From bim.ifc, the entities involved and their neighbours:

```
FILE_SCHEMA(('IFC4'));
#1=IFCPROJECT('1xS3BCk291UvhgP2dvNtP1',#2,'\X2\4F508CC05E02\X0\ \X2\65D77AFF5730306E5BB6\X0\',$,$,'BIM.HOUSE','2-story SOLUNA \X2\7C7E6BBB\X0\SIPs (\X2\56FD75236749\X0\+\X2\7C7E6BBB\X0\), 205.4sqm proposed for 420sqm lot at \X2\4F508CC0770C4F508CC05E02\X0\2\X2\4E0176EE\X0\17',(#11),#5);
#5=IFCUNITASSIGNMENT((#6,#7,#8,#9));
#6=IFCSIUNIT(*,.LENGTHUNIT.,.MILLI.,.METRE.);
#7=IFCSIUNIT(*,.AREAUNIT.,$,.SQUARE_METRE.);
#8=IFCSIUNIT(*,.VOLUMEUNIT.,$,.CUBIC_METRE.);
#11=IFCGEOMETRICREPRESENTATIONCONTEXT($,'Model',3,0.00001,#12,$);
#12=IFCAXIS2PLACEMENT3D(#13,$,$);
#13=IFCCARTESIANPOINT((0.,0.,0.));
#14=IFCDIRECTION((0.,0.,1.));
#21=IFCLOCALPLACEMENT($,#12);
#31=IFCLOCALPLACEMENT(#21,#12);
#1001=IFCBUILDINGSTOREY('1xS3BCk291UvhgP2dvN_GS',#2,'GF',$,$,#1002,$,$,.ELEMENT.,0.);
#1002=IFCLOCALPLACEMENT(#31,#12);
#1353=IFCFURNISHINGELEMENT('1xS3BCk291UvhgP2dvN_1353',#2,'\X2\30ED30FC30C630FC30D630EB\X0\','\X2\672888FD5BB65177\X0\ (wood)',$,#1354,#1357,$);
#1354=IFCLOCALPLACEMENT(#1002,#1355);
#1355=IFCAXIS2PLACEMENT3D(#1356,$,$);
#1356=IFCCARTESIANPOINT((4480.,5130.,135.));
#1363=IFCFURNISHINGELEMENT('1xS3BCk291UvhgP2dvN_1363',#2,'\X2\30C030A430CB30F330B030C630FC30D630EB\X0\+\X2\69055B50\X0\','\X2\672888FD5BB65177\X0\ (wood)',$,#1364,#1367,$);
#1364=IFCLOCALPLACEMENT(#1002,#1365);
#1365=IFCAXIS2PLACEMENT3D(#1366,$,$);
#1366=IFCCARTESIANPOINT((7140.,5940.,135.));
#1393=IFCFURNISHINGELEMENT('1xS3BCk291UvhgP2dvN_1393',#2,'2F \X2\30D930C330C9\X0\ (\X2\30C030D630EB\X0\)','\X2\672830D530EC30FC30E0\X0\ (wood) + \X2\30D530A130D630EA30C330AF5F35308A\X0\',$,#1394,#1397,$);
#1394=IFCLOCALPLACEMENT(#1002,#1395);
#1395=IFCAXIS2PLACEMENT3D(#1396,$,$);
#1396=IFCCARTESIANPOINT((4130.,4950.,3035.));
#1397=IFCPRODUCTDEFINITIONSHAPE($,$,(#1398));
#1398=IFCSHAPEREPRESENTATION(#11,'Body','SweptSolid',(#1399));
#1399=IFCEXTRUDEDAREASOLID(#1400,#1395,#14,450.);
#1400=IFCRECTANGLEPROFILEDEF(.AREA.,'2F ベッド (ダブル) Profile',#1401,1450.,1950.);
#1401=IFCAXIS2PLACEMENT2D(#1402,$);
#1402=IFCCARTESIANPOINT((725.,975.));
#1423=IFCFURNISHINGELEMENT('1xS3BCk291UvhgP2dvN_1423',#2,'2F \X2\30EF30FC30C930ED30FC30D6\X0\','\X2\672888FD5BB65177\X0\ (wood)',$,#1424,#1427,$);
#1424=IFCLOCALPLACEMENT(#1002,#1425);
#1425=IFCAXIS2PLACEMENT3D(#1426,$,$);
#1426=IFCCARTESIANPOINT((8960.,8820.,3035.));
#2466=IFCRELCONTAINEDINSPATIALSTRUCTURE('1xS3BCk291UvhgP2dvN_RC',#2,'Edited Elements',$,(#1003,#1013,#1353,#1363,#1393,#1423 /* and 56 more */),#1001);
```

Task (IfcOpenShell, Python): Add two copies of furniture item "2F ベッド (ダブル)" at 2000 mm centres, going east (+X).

```python
import numpy as np
import ifcopenshell
import ifcopenshell.api.geometry
import ifcopenshell.api.root
import ifcopenshell.util.element
import ifcopenshell.util.placement

model = ifcopenshell.open("bim.ifc")


def reuse_history(source, copy):
    """copy_class also copies each property set's owner history, people and application; keep the originals."""
    for rel in copy.IsDefinedBy:
        if rel.is_a("IfcRelDefinesByProperties") and (history := rel.RelatingPropertyDefinition.OwnerHistory):
            rel.RelatingPropertyDefinition.OwnerHistory = source.OwnerHistory
            ifcopenshell.util.element.remove_deep2(model, history)


source = model.by_guid("1xS3BCk291UvhgP2dvN_1393")
base = ifcopenshell.util.placement.get_local_placement(source.ObjectPlacement)
step = np.array([1.0, 0.0, 0.0]) * 2000.0

for i in range(1, 3):
    copy = ifcopenshell.api.root.copy_class(model, product=source)
    copy.Representation = ifcopenshell.util.element.copy_deep(
        model, source.Representation, exclude=["IfcGeometricRepresentationContext", "IfcRepresentationMap"]
    )
    reuse_history(source, copy)
    matrix = base.copy()
    matrix[:3, 3] += i * step
    print("added at", matrix[:3, 3].round(3) + 0.0)
    ifcopenshell.api.geometry.edit_object_placement(model, product=copy, matrix=matrix, is_si=False)

model.write("bim_edited.ifc")
```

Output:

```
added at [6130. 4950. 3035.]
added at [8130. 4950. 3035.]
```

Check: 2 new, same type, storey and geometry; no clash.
